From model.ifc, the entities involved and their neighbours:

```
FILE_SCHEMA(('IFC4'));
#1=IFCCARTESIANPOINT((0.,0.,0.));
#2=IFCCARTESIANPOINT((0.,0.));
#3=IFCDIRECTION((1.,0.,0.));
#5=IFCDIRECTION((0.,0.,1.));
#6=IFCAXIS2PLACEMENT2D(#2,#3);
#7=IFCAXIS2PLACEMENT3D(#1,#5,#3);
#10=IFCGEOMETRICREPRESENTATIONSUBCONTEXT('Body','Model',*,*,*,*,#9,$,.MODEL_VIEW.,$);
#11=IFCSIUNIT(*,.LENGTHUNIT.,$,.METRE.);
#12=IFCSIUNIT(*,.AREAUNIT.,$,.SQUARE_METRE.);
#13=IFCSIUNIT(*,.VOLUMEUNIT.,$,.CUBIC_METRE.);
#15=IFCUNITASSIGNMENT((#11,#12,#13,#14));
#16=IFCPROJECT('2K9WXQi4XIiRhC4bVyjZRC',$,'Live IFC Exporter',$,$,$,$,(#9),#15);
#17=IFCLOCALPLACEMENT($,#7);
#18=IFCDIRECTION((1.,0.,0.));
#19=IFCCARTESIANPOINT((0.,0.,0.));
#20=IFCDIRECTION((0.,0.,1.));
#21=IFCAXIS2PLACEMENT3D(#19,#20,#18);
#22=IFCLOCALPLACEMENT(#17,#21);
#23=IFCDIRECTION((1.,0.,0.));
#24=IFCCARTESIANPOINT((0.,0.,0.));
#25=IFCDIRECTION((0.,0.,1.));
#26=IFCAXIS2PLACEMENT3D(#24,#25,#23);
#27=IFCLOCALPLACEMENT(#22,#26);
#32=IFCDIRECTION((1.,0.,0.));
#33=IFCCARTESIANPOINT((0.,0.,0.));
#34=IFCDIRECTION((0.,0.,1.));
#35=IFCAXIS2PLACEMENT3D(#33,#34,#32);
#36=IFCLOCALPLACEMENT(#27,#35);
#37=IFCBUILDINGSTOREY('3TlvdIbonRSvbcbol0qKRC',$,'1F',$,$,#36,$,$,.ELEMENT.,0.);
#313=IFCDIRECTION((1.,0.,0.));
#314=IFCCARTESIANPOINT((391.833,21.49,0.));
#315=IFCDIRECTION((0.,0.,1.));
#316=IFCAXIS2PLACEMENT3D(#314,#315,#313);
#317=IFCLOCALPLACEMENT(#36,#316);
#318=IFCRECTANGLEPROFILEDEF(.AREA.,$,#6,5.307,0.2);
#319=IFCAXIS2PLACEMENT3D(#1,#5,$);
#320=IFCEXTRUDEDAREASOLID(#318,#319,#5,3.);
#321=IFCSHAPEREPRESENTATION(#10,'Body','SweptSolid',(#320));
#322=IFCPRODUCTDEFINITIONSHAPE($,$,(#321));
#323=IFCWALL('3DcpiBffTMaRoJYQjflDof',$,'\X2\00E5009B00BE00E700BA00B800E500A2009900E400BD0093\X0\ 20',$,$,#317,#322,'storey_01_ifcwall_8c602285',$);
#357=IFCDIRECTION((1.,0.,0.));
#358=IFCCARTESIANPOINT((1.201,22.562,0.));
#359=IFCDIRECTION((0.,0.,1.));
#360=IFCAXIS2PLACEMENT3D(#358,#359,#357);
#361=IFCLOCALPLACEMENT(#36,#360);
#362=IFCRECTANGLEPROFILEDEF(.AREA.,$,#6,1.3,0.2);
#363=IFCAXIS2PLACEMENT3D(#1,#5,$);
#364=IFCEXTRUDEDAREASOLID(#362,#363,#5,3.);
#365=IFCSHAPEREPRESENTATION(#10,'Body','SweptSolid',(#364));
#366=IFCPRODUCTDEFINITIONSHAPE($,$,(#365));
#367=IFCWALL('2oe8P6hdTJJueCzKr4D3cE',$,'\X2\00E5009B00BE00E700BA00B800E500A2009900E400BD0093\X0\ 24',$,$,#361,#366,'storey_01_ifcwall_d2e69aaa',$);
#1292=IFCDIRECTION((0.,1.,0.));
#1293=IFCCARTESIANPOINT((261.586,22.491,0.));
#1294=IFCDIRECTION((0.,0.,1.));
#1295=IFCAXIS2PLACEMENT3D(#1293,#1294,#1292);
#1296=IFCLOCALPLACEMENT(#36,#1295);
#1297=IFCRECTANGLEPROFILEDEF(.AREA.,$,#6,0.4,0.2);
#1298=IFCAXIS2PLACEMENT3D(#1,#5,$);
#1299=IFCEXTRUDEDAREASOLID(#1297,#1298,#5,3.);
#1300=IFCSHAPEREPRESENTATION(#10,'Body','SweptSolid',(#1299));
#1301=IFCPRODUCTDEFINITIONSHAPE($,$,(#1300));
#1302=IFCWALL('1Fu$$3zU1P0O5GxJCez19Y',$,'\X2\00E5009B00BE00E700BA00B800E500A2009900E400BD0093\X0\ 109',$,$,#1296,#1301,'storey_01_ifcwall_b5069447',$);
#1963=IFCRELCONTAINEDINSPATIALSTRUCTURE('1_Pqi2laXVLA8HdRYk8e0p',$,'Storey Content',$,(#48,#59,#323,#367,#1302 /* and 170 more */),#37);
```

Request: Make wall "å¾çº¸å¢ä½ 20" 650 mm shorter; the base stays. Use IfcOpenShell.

```python
import ifcopenshell
import ifcopenshell.geom
import ifcopenshell.util.representation
import ifcopenshell.util.shape
import ifcopenshell.util.unit

model = ifcopenshell.open("model.ifc")
unit_scale = ifcopenshell.util.unit.calculate_unit_scale(model)
settings = ifcopenshell.geom.settings()


def volume(element):
    """Net volume in cubic metres, openings subtracted."""
    shape = ifcopenshell.geom.create_shape(settings, element)
    return ifcopenshell.util.shape.get_volume(shape.geometry)


wall = model.by_guid("3DcpiBffTMaRoJYQjflDof")
before = volume(wall)

body = ifcopenshell.util.representation.get_representation(wall, "Model", "Body")
solid = body.Items[0]
old_height = solid.Depth
solid.Depth -= 0.65 / unit_scale
after = volume(wall)

print(f"height {old_height:g} -> {solid.Depth:g}, volume {before:.3f} -> {after:.3f} m3")

model.write("model_rev.ifc")
```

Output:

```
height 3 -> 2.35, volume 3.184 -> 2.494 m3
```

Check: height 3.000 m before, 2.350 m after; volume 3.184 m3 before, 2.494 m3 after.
